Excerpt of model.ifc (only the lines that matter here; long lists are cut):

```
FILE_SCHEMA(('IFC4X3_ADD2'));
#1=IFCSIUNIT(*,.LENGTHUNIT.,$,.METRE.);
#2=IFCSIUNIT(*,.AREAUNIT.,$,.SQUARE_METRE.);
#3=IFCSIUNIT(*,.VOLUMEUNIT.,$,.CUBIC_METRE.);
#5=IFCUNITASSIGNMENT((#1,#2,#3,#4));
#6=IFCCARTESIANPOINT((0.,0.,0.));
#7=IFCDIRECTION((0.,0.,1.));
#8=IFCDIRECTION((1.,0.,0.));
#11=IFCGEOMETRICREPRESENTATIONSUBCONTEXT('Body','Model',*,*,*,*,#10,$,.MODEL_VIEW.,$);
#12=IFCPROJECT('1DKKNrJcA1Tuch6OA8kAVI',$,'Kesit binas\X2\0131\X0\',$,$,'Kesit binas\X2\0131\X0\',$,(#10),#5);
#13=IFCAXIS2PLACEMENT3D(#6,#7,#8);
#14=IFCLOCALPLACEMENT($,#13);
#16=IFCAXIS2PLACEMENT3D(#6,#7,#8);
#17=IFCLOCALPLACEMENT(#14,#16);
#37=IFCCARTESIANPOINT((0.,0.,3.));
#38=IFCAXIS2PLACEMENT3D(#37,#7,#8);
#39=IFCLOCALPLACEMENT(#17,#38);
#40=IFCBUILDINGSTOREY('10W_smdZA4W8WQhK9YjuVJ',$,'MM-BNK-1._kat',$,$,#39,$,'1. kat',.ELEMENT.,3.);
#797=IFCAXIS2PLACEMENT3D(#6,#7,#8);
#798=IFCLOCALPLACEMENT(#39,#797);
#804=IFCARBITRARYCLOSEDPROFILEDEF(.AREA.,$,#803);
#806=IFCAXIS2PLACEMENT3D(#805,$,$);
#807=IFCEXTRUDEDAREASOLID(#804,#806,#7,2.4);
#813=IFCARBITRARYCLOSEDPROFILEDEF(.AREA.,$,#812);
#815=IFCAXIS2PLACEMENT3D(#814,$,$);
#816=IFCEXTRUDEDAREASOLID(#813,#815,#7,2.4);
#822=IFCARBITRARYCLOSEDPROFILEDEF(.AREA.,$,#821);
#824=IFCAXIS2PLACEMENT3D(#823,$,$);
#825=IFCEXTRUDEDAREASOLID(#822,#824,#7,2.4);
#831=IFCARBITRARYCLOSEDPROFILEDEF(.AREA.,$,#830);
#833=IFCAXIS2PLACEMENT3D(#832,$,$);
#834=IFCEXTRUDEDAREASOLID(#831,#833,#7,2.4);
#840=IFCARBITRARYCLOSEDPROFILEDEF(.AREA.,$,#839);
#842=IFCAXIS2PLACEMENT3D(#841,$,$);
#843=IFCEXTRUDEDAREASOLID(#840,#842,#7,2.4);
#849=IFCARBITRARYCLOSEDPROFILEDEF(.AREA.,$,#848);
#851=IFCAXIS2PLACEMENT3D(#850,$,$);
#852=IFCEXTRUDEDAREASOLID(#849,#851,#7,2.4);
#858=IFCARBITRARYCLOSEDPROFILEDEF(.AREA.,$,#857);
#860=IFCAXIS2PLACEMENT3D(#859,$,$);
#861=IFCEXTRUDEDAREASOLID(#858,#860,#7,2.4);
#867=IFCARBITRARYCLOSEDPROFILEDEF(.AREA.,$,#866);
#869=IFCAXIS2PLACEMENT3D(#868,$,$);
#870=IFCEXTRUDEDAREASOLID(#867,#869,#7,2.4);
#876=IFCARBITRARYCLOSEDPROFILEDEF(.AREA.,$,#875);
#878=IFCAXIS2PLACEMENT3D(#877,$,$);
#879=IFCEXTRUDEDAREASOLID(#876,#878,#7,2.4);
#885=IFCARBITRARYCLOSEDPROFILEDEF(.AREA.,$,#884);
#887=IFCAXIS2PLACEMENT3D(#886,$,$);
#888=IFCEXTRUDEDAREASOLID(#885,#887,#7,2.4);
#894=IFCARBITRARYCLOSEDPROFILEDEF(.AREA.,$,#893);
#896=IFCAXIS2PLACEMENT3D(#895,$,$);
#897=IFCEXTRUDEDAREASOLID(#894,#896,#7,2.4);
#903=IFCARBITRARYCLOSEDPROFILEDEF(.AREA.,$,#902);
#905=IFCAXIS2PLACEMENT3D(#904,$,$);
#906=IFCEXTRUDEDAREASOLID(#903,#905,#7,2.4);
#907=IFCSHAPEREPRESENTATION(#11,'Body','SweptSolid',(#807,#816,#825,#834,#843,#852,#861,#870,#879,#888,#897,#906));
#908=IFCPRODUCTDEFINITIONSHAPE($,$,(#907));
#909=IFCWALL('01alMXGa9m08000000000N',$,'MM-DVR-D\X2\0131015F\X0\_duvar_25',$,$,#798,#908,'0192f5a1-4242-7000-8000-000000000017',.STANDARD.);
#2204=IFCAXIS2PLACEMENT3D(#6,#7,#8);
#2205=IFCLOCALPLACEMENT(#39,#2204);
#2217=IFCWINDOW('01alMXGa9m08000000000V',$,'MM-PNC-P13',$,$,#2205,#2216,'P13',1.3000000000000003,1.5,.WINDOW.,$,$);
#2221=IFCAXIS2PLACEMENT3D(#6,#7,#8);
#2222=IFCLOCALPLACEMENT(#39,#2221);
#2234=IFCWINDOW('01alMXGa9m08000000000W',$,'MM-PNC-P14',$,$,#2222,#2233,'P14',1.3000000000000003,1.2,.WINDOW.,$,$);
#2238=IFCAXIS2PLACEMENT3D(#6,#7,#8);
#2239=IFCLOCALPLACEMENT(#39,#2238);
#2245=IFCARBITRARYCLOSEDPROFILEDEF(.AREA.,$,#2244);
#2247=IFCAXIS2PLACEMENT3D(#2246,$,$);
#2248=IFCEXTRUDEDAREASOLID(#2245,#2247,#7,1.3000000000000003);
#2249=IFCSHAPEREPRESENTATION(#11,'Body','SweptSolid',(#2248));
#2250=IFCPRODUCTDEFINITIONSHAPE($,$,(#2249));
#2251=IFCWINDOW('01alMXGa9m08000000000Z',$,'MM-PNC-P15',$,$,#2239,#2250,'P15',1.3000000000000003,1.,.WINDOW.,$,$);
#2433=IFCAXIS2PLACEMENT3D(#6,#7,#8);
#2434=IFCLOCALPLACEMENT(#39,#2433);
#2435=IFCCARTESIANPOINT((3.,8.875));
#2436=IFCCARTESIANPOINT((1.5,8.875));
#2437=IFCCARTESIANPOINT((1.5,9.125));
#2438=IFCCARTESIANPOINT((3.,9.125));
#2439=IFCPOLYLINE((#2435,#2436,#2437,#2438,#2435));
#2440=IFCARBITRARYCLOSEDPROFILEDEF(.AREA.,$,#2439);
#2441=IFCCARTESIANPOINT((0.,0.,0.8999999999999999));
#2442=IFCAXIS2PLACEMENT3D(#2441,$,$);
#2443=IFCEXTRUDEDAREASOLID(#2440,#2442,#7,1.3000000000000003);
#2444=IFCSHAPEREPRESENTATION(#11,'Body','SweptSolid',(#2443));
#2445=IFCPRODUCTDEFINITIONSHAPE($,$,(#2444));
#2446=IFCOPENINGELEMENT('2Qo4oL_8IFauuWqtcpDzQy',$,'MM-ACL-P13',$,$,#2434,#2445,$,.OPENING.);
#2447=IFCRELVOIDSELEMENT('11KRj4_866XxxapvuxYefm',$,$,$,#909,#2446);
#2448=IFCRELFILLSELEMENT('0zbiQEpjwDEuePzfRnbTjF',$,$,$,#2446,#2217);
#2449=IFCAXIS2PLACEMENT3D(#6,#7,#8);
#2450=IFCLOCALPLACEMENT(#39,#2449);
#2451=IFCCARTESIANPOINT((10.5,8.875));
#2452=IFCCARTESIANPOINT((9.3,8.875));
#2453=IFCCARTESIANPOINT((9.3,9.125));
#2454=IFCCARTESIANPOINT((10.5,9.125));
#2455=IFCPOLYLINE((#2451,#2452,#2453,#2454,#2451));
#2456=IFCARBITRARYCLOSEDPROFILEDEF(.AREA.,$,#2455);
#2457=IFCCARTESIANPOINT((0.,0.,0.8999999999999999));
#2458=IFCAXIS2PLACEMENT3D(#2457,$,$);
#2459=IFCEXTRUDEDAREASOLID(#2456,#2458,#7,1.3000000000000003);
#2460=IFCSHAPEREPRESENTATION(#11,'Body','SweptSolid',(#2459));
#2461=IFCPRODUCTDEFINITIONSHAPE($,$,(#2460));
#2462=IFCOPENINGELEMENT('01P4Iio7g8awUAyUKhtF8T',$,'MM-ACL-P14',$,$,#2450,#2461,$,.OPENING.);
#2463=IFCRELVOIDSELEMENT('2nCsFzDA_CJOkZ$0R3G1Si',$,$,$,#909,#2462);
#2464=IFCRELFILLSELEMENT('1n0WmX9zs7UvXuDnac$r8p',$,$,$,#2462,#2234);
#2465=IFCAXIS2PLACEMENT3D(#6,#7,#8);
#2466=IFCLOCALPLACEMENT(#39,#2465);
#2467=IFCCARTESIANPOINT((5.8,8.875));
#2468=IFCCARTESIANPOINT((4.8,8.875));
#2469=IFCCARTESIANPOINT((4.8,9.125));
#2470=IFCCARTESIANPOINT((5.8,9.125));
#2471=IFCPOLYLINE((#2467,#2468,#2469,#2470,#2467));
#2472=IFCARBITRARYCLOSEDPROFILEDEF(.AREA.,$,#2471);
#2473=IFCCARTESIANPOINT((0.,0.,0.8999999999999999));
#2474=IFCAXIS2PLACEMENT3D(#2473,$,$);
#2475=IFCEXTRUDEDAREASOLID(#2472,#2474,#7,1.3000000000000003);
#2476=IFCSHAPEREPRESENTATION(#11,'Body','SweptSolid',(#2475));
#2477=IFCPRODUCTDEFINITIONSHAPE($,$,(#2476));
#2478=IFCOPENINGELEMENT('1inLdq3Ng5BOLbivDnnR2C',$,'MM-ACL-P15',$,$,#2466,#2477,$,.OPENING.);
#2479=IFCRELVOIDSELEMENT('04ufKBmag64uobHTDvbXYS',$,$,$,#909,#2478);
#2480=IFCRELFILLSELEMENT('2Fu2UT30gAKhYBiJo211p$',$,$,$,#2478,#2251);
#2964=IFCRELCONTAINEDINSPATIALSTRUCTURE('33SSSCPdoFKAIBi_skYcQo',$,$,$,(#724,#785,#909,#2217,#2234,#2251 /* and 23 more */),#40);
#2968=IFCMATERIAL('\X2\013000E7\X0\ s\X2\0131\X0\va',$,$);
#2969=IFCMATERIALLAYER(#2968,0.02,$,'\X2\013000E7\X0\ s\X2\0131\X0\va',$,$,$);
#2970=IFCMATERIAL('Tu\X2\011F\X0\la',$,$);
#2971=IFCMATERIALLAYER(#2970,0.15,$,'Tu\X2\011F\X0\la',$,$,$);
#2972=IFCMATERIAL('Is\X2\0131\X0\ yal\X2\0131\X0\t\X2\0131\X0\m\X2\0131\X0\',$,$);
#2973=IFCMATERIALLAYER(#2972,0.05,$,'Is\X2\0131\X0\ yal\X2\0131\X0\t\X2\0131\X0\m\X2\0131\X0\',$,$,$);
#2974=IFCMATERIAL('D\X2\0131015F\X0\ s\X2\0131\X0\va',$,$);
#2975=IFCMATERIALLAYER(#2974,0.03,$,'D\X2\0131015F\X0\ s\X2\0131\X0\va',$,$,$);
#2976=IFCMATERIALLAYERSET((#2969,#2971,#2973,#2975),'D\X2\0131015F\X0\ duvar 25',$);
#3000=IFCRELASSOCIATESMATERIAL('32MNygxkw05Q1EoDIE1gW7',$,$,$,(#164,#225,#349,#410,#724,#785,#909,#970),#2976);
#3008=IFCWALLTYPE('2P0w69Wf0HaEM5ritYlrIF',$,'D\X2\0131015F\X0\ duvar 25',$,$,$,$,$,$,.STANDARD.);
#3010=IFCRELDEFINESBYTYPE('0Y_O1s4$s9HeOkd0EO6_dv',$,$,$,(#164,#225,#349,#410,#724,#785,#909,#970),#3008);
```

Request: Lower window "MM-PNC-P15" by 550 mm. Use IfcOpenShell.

```python
import numpy as np
import ifcopenshell
import ifcopenshell.api.geometry
import ifcopenshell.util.placement
import ifcopenshell.util.unit

model = ifcopenshell.open("model.ifc")
unit_scale = ifcopenshell.util.unit.calculate_unit_scale(model)

window = model.by_guid("01alMXGa9m08000000000Z")
opening = window.FillsVoids[0].RelatingOpeningElement
dz = -0.55

shift = np.array([0.0, 0.0, dz])
# The window is not placed relative to its opening, so move both.
for product in (opening, window):
    matrix = ifcopenshell.util.placement.get_local_placement(product.ObjectPlacement)
    matrix[:3, 3] += shift
    ifcopenshell.api.geometry.edit_object_placement(model, product=product, matrix=matrix, is_si=False)

print(f"moved by {dz * unit_scale:+.3f} m")

model.write("model_rev.ifc")
```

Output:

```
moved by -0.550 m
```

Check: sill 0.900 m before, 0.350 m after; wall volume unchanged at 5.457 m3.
